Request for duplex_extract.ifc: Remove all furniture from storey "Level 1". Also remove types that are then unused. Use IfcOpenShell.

First a look at what the model holds.

```python
import ifcopenshell
import ifcopenshell.util.element

model = ifcopenshell.open("duplex_extract.ifc")
print(model.schema)
storey = next(s for s in model.by_type("IfcBuildingStorey") if s.Name == "Level 1")
furniture = [e for e in ifcopenshell.util.element.get_decomposition(storey) if e.is_a("IfcFurnishingElement")]
seen = {}
for e in furniture:
    element_type = ifcopenshell.util.element.get_type(e)
    name = element_type.Name if element_type not in (None, e) else None
    seen[name] = seen.get(name, 0) + 1
for name, count in sorted(seen.items(), key=str):
    print(count, "x", name)
```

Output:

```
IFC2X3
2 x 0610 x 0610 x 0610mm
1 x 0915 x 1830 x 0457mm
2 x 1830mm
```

```python
import ifcopenshell
import ifcopenshell.api.root
import ifcopenshell.util.element

model = ifcopenshell.open("duplex_extract.ifc")

storey = next(s for s in model.by_type("IfcBuildingStorey") if s.Name == "Level 1")
furniture = [e for e in ifcopenshell.util.element.get_decomposition(storey) if e.is_a("IfcFurnishingElement")]
types = {ifcopenshell.util.element.get_type(e) for e in furniture} - {None, *furniture}

for e in furniture:
    ifcopenshell.api.root.remove_product(model, product=e)
print(len(furniture), "removed")

unused = [t for t in types if not ifcopenshell.util.element.get_types(t)]
for t in unused:
    ifcopenshell.api.root.remove_product(model, product=t)
print(len(unused), "unused types removed")

model.write("duplex_extract_updated.ifc")
```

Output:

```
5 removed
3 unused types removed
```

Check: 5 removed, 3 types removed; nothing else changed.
